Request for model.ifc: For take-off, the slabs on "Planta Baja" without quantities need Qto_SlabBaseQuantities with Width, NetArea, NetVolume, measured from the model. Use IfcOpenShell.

First a look at what the model holds.

```python
import ifcopenshell
import ifcopenshell.util.element
import ifcopenshell.util.unit

model = ifcopenshell.open("model.ifc")
print(model.schema)
for unit_type in ("LENGTHUNIT", "AREAUNIT", "VOLUMEUNIT"):
    print(unit_type, ifcopenshell.util.unit.calculate_unit_scale(model, unit_type))
storey = next(s for s in model.by_type("IfcBuildingStorey") if s.Name == "Planta Baja")
slabs = [e for e in ifcopenshell.util.element.get_decomposition(storey) if e.is_a("IfcSlab")]
for e in sorted(slabs, key=lambda e: e.id()):
    print(e.id(), e.is_a(), e.Name, list(ifcopenshell.util.element.get_psets(e, qtos_only=True)), sep=" | ")
```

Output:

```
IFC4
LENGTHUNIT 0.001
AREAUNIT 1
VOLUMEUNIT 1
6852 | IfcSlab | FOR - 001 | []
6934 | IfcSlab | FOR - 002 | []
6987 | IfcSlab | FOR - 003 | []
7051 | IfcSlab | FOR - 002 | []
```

```python
import ifcopenshell
import ifcopenshell.api.pset
import ifcopenshell.geom
import ifcopenshell.util.element
import ifcopenshell.util.shape
import ifcopenshell.util.unit

model = ifcopenshell.open("model.ifc")
unit_scale = ifcopenshell.util.unit.calculate_unit_scale(model)
area_scale = ifcopenshell.util.unit.calculate_unit_scale(model, "AREAUNIT")
volume_scale = ifcopenshell.util.unit.calculate_unit_scale(model, "VOLUMEUNIT")
settings = ifcopenshell.geom.settings()

storey = next(s for s in model.by_type("IfcBuildingStorey") if s.Name == "Planta Baja")
slabs = [e for e in ifcopenshell.util.element.get_decomposition(storey) if e.is_a("IfcSlab")]

for e in sorted(slabs, key=lambda e: e.id()):
    if ifcopenshell.util.element.get_psets(e, qtos_only=True, should_inherit=False):
        continue
    # Geometry comes back in metres, in the element's own axes.
    shape = ifcopenshell.geom.create_shape(settings, e)
    values = {
        "Width": ifcopenshell.util.shape.get_z(shape.geometry) / unit_scale,
        "NetArea": ifcopenshell.util.shape.get_footprint_area(shape.geometry) / area_scale,
        "NetVolume": ifcopenshell.util.shape.get_volume(shape.geometry) / volume_scale,
    }
    qto = ifcopenshell.api.pset.add_qto(model, product=e, name="Qto_SlabBaseQuantities")
    ifcopenshell.api.pset.edit_qto(model, qto=qto, properties=values)
    print(e.id(), {k: round(v, 3) for k, v in values.items()})

model.write("model_v2.ifc")
```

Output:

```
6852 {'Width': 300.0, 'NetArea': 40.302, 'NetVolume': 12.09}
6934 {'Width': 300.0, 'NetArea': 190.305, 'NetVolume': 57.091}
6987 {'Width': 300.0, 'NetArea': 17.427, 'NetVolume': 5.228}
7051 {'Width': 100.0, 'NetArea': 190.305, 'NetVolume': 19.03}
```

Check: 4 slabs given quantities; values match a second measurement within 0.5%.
